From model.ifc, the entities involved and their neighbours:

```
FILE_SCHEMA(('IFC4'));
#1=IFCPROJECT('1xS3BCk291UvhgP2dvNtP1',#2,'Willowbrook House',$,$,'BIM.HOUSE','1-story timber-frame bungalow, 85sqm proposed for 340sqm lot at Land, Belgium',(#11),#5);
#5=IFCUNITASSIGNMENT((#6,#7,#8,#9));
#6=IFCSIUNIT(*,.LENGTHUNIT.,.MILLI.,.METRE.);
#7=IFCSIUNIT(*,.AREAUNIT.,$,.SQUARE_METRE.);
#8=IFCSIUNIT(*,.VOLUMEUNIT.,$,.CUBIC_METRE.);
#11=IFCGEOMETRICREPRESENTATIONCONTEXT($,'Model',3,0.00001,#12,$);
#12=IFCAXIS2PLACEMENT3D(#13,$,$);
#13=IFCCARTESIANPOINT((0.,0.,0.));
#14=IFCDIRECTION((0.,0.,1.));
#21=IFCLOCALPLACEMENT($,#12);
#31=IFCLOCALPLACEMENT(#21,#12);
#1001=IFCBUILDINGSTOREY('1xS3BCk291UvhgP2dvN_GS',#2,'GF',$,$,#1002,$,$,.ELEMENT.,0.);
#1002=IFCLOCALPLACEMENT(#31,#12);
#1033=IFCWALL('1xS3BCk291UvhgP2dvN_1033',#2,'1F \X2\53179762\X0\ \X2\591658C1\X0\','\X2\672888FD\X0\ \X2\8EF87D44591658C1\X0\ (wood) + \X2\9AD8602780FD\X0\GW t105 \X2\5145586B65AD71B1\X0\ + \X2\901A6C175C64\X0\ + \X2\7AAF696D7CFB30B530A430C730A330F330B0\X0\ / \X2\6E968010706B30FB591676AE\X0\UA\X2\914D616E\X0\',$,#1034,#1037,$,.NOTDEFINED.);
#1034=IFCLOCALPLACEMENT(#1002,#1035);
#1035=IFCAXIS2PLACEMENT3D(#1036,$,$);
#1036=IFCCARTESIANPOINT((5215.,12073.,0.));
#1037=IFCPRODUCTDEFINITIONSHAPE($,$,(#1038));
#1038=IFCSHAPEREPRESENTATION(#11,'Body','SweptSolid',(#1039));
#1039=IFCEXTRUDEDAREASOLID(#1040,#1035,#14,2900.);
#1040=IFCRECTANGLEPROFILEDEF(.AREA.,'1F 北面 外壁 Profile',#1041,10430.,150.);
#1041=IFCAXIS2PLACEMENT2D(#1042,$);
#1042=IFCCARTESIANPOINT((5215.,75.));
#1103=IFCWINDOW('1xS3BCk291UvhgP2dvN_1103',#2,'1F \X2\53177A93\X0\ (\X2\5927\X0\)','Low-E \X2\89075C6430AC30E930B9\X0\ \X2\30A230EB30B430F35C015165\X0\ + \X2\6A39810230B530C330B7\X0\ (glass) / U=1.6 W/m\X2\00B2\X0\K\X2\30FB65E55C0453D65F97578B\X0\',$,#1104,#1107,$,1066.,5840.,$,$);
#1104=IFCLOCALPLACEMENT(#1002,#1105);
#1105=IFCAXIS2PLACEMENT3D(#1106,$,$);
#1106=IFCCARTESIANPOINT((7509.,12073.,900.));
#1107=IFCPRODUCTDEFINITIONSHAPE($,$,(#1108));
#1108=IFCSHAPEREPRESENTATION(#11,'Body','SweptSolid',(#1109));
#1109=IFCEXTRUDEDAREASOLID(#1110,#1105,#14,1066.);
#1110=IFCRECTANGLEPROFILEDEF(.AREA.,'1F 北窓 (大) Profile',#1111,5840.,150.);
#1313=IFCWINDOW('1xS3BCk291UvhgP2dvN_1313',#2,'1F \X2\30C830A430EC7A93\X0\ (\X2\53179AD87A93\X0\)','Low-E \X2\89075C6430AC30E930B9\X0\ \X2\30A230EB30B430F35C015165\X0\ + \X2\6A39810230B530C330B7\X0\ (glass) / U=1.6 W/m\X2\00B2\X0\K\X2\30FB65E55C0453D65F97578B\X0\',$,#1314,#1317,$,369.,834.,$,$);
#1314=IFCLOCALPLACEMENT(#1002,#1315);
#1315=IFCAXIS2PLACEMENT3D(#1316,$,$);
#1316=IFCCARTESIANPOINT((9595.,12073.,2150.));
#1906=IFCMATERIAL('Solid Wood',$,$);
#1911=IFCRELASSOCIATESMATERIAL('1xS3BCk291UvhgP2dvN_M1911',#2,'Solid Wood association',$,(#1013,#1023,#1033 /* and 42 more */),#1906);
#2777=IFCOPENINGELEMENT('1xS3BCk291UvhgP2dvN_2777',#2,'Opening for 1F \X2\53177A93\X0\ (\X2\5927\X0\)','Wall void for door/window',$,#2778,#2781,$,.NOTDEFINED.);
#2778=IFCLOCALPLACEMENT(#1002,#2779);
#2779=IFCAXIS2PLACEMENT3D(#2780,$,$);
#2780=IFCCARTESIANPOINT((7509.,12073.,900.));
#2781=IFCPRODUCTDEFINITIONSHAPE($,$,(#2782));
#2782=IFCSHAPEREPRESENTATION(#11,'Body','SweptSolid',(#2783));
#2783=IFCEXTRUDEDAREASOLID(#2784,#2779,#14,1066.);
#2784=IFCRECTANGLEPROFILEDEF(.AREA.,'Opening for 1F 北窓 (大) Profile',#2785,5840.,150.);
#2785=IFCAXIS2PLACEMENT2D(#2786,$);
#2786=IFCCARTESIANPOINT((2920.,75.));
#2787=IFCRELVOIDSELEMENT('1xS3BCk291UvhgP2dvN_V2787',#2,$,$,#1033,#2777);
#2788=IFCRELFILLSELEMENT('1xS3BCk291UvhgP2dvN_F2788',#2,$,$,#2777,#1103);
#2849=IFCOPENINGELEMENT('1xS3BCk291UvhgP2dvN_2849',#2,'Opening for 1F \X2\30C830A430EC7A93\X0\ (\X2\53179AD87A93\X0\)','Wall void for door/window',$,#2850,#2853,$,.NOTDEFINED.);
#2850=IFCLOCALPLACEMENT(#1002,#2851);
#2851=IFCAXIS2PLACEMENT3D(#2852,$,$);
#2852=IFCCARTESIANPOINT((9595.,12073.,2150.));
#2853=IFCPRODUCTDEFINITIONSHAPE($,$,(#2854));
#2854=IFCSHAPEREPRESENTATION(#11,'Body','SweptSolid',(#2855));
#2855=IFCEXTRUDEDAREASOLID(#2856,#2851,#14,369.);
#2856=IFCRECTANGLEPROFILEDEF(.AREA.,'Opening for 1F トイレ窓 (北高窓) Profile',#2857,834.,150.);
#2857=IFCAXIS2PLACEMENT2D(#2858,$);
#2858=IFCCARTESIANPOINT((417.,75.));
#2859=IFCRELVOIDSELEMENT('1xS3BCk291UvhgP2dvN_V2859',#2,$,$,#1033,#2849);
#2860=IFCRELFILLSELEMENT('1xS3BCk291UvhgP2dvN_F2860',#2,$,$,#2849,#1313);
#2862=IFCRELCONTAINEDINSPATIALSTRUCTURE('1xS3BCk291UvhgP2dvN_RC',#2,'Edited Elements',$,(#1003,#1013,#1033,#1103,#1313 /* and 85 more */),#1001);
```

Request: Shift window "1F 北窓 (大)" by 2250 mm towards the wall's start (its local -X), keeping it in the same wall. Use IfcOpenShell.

```python
import ifcopenshell
import ifcopenshell.api.geometry
import ifcopenshell.util.placement
import ifcopenshell.util.unit

model = ifcopenshell.open("model.ifc")
unit_scale = ifcopenshell.util.unit.calculate_unit_scale(model)

window = model.by_guid("1xS3BCk291UvhgP2dvN_1103")
opening = window.FillsVoids[0].RelatingOpeningElement
wall = opening.VoidsElements[0].RelatingBuildingElement

wall_matrix = ifcopenshell.util.placement.get_local_placement(wall.ObjectPlacement)
shift = wall_matrix[:3, 0] * -2.25 / unit_scale
before = ifcopenshell.util.placement.get_local_placement(window.ObjectPlacement)[:3, 3].copy()

# The window is not placed relative to its opening, so move both.
for product in (opening, window):
    matrix = ifcopenshell.util.placement.get_local_placement(product.ObjectPlacement)
    matrix[:3, 3] += shift
    ifcopenshell.api.geometry.edit_object_placement(model, product=product, matrix=matrix, is_si=False)

after = ifcopenshell.util.placement.get_local_placement(window.ObjectPlacement)[:3, 3]
print("window moved by", (after - before).round(3) + 0.0)

model.write("model_updated.ifc")
```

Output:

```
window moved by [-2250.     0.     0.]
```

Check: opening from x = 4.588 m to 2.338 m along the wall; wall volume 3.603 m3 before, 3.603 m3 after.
